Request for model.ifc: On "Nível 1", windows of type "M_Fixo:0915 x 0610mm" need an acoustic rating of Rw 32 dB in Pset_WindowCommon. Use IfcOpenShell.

First a look at what the model holds.

```python
import ifcopenshell
import ifcopenshell.util.element

model = ifcopenshell.open("model.ifc")
print(model.schema)
storey = next(s for s in model.by_type("IfcBuildingStorey") if s.Name == "Nível 1")
windows = [e for e in ifcopenshell.util.element.get_decomposition(storey) if e.is_a("IfcWindow")]
seen = {}
for e in windows:
    element_type = ifcopenshell.util.element.get_type(e)
    key = (element_type.Name if element_type != e and element_type else None, ifcopenshell.util.element.get_pset(e, "Pset_WindowCommon", "AcousticRating"))
    seen[key] = seen.get(key, 0) + 1
for (name, value), count in sorted(seen.items(), key=str):
    print(count, "x", name, "|", value)
```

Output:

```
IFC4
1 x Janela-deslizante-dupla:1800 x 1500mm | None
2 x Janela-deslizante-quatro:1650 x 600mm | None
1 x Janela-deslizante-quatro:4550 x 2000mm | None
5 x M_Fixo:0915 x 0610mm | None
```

```python
import ifcopenshell
import ifcopenshell.api.pset
import ifcopenshell.util.element

model = ifcopenshell.open("model.ifc")

storey = next(s for s in model.by_type("IfcBuildingStorey") if s.Name == "Nível 1")
windows = [e for e in ifcopenshell.util.element.get_decomposition(storey) if e.is_a("IfcWindow")]

count = 0
for e in windows:
    element_type = ifcopenshell.util.element.get_type(e)
    if element_type in (None, e) or element_type.Name != "M_Fixo:0915 x 0610mm":
        continue
    # add_pset returns the element's existing set when there is one.
    pset = ifcopenshell.api.pset.add_pset(model, product=e, name="Pset_WindowCommon")
    ifcopenshell.api.pset.edit_pset(model, pset=pset, properties={"AcousticRating": "Rw 32 dB"})
    count += 1

print(count, "windows updated")

model.write("model-out.ifc")
```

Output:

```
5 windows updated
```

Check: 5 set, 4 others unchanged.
